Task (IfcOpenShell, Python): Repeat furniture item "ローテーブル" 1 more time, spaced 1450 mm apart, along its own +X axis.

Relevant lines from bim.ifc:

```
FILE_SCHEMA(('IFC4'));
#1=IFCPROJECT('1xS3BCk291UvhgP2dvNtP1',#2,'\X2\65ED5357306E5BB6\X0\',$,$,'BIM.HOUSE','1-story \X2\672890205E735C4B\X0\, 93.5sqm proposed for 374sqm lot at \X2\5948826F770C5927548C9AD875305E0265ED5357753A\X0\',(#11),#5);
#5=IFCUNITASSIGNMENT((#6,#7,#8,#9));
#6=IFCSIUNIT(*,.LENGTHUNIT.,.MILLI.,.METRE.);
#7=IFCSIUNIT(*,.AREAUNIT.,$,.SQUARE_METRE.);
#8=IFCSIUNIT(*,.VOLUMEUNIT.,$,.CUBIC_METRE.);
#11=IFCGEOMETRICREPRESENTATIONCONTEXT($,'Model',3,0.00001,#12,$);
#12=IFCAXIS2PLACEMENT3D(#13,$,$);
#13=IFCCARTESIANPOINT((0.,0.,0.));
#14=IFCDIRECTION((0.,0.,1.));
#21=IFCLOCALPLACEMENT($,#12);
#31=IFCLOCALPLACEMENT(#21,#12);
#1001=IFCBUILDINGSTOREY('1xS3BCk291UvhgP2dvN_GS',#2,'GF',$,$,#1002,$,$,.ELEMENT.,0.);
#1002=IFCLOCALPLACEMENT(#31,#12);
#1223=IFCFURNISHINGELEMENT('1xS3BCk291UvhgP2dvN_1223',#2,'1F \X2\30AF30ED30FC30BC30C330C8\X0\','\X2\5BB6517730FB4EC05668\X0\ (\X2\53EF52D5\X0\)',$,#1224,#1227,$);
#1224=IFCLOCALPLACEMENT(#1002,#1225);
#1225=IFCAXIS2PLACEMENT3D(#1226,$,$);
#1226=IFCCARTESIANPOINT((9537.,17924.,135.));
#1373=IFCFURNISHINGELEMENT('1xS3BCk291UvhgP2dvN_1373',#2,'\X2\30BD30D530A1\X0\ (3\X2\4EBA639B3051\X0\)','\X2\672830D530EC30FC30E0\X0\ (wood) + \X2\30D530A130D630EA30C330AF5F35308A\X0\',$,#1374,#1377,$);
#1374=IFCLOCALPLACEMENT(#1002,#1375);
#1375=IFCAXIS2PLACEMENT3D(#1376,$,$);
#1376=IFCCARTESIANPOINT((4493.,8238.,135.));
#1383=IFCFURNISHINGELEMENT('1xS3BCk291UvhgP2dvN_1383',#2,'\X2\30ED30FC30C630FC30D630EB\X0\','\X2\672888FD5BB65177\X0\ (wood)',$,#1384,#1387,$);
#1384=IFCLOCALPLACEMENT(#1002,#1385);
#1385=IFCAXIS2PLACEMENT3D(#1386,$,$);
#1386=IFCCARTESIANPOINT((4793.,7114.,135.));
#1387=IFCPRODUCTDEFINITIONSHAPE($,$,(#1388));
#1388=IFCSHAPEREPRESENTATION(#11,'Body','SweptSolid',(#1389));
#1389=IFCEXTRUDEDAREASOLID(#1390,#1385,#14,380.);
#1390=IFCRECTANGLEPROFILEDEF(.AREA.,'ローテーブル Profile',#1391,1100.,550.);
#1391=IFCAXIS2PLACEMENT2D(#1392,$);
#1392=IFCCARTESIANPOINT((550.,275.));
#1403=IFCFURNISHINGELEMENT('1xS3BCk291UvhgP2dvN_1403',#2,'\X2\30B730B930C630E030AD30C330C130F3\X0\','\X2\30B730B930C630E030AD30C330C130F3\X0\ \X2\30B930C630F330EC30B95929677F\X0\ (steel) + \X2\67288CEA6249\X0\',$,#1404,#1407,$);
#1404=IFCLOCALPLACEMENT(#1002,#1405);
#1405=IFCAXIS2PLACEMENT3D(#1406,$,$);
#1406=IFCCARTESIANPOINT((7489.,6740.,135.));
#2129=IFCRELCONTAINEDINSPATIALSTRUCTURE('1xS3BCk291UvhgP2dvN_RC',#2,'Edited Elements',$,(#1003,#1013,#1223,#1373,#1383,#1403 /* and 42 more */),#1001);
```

```python
import ifcopenshell
import ifcopenshell.api.geometry
import ifcopenshell.api.root
import ifcopenshell.util.element
import ifcopenshell.util.placement
import ifcopenshell.util.unit

model = ifcopenshell.open("bim.ifc")
unit_scale = ifcopenshell.util.unit.calculate_unit_scale(model)


def reuse_history(source, copy):
    """copy_class also copies each property set's owner history, people and application; keep the originals."""
    for rel in copy.IsDefinedBy:
        if rel.is_a("IfcRelDefinesByProperties") and (history := rel.RelatingPropertyDefinition.OwnerHistory):
            rel.RelatingPropertyDefinition.OwnerHistory = source.OwnerHistory
            ifcopenshell.util.element.remove_deep2(model, history)


source = model.by_guid("1xS3BCk291UvhgP2dvN_1383")
base = ifcopenshell.util.placement.get_local_placement(source.ObjectPlacement)
step = base[:3, 0] * 1.45 / unit_scale

for i in range(1, 2):
    copy = ifcopenshell.api.root.copy_class(model, product=source)
    copy.Representation = ifcopenshell.util.element.copy_deep(
        model, source.Representation, exclude=["IfcGeometricRepresentationContext", "IfcRepresentationMap"]
    )
    reuse_history(source, copy)
    matrix = base.copy()
    matrix[:3, 3] += i * step
    print("added at", matrix[:3, 3].round(3) + 0.0)
    ifcopenshell.api.geometry.edit_object_placement(model, product=copy, matrix=matrix, is_si=False)

model.write("bim_edited.ifc")
```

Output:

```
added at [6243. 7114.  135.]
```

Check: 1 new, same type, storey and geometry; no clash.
